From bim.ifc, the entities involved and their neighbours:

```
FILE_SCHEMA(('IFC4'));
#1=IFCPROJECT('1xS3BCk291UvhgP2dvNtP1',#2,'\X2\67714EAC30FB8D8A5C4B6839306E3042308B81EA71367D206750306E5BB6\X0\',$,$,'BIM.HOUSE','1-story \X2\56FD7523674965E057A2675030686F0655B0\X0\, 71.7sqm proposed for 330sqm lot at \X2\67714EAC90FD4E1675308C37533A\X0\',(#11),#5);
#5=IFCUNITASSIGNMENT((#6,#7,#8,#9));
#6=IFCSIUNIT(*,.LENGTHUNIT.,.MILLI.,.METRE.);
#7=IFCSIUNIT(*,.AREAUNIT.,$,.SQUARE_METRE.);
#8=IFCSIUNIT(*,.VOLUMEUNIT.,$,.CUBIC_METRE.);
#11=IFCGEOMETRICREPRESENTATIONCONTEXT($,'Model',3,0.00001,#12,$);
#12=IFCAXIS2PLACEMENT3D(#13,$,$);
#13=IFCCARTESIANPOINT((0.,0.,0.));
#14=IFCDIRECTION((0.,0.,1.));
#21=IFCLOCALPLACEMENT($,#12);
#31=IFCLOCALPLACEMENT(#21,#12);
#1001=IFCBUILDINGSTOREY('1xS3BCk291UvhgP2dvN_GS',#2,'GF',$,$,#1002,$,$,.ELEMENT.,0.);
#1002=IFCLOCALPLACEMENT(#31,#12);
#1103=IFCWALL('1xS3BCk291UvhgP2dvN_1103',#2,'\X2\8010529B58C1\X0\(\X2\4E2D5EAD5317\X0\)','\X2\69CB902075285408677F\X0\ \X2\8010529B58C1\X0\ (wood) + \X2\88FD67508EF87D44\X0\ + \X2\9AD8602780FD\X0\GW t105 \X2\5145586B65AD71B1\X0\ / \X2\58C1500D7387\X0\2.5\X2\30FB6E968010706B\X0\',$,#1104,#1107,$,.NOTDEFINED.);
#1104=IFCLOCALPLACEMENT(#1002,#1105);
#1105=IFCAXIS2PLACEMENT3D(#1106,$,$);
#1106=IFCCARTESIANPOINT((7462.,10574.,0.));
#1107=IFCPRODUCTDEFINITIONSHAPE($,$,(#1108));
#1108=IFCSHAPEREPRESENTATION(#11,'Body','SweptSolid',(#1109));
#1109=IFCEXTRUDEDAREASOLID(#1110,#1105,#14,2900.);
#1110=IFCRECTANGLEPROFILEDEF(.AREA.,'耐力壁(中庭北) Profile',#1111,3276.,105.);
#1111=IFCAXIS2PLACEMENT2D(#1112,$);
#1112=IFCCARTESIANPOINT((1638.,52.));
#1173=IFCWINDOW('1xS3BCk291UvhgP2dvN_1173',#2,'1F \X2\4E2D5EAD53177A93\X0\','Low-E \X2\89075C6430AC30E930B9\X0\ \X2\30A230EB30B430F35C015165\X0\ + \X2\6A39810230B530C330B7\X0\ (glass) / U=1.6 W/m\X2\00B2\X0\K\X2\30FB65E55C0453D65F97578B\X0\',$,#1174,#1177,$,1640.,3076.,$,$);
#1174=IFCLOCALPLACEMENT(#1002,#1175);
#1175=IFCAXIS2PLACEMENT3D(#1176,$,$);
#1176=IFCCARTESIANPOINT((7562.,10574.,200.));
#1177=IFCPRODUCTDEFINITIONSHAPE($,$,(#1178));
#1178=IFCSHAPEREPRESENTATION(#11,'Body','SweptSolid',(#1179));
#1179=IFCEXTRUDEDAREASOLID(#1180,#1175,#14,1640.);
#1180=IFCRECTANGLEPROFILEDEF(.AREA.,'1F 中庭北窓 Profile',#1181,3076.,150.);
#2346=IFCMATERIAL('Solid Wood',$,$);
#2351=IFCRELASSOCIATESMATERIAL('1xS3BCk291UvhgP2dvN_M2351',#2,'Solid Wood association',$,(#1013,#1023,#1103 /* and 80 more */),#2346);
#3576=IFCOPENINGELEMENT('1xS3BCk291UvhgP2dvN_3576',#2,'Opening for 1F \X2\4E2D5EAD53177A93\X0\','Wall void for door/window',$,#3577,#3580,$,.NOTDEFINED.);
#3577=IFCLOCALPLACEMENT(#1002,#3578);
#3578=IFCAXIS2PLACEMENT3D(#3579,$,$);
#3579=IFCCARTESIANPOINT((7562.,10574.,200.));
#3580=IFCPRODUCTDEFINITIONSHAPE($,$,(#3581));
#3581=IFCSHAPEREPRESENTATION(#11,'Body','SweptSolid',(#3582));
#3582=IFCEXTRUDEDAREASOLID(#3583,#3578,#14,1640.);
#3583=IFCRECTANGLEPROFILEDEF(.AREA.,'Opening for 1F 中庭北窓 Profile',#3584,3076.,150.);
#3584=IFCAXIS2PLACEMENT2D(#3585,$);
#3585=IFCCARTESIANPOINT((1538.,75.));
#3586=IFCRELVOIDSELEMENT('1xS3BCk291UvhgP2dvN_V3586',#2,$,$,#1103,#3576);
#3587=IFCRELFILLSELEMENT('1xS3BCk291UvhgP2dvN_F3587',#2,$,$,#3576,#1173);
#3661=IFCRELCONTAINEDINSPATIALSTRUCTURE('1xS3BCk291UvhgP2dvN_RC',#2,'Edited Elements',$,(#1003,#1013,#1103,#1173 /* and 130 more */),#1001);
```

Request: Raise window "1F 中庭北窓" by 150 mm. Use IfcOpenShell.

```python
import numpy as np
import ifcopenshell
import ifcopenshell.api.geometry
import ifcopenshell.util.placement
import ifcopenshell.util.unit

model = ifcopenshell.open("bim.ifc")
unit_scale = ifcopenshell.util.unit.calculate_unit_scale(model)

window = model.by_guid("1xS3BCk291UvhgP2dvN_1173")
opening = window.FillsVoids[0].RelatingOpeningElement
dz = 0.15 / unit_scale

shift = np.array([0.0, 0.0, dz])
# The window is not placed relative to its opening, so move both.
for product in (opening, window):
    matrix = ifcopenshell.util.placement.get_local_placement(product.ObjectPlacement)
    matrix[:3, 3] += shift
    ifcopenshell.api.geometry.edit_object_placement(model, product=product, matrix=matrix, is_si=False)

print(f"moved by {dz * unit_scale:+.3f} m")

model.write("bim_updated.ifc")
```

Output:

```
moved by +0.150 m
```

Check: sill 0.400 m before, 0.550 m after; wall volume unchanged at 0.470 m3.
